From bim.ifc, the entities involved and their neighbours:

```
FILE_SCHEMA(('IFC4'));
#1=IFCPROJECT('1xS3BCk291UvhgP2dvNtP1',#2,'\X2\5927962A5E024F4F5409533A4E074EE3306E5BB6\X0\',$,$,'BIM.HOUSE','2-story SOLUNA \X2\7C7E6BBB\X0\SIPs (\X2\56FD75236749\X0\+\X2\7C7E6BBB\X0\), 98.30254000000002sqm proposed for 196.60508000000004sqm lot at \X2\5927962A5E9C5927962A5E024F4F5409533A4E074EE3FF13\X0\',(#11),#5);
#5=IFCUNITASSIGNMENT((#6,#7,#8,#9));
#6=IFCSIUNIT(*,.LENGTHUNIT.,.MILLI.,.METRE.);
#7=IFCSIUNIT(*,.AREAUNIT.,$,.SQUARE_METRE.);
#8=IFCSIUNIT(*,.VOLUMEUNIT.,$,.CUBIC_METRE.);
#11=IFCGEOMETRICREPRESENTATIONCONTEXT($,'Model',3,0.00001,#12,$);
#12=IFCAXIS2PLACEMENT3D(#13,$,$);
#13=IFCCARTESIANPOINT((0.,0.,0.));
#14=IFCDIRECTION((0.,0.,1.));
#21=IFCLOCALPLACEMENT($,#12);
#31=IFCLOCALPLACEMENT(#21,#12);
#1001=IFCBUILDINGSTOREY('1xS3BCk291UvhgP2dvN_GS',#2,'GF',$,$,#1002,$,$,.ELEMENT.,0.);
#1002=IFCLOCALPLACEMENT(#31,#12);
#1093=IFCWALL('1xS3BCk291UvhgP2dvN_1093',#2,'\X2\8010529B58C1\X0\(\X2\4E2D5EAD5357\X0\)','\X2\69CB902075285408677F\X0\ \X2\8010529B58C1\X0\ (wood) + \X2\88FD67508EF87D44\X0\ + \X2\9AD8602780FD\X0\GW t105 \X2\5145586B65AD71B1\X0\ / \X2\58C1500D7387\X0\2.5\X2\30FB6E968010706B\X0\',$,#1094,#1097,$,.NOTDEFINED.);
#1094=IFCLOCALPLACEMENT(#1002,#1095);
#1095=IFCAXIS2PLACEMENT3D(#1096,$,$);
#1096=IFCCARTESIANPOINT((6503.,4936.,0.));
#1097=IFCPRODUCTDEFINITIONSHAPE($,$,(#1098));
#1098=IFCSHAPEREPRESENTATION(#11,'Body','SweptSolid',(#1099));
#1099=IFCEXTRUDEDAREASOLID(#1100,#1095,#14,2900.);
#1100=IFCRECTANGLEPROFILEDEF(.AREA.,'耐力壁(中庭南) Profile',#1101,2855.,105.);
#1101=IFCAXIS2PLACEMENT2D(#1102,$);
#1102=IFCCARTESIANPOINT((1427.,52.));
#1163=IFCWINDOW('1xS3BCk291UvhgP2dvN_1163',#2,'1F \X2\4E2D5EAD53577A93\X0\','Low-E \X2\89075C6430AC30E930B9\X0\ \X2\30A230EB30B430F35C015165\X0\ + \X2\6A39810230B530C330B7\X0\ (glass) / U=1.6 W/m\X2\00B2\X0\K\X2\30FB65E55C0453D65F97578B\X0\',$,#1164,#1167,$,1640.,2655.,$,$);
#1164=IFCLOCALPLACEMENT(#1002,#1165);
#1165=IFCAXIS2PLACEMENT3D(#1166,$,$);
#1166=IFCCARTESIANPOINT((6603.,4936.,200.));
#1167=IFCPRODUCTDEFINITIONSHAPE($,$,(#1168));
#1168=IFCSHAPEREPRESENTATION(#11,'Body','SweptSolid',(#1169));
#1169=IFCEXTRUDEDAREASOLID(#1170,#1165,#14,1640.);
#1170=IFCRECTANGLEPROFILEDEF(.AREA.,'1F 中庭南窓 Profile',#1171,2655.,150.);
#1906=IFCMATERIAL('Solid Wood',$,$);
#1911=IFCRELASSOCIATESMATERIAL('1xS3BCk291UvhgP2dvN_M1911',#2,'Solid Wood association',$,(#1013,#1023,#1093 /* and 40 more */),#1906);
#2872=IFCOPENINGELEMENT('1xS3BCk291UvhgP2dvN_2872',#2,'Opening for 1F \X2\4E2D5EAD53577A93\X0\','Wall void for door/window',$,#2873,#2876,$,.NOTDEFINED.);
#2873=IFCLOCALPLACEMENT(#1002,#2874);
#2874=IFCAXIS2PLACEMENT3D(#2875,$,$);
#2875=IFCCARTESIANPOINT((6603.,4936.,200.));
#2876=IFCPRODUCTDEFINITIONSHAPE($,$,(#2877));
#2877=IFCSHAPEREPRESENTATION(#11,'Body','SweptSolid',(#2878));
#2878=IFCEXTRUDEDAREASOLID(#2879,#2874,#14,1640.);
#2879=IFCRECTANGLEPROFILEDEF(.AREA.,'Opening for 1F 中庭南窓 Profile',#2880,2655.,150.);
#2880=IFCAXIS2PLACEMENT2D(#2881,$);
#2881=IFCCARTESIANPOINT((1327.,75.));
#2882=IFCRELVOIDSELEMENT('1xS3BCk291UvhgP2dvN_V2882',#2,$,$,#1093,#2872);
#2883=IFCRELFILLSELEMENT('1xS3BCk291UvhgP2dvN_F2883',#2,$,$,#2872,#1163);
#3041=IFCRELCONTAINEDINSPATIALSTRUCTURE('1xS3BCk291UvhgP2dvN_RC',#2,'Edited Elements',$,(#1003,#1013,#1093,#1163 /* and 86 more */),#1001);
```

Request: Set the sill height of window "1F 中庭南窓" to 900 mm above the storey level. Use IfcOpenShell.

```python
import numpy as np
import ifcopenshell
import ifcopenshell.api.geometry
import ifcopenshell.geom
import ifcopenshell.util.element
import ifcopenshell.util.placement
import ifcopenshell.util.shape
import ifcopenshell.util.unit

model = ifcopenshell.open("bim.ifc")
unit_scale = ifcopenshell.util.unit.calculate_unit_scale(model)

window = model.by_guid("1xS3BCk291UvhgP2dvN_1163")
opening = window.FillsVoids[0].RelatingOpeningElement
storey = ifcopenshell.util.element.get_container(window, ifc_class="IfcBuildingStorey")
level = ifcopenshell.util.placement.get_local_placement(storey.ObjectPlacement)[2, 3]

# The opening's origin need not be at the sill, so measure its lowest point.
shape = ifcopenshell.geom.create_shape(ifcopenshell.geom.settings(), opening)
bottom = ifcopenshell.util.shape.get_shape_bottom_elevation(shape, shape.geometry) / unit_scale
dz = level + 900.0 - bottom

shift = np.array([0.0, 0.0, dz])
# The window is not placed relative to its opening, so move both.
for product in (opening, window):
    matrix = ifcopenshell.util.placement.get_local_placement(product.ObjectPlacement)
    matrix[:3, 3] += shift
    ifcopenshell.api.geometry.edit_object_placement(model, product=product, matrix=matrix, is_si=False)

print(f"moved by {dz * unit_scale:+.3f} m")

model.write("bim_edited.ifc")
```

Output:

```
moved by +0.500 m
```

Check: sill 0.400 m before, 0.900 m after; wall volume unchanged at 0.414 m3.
